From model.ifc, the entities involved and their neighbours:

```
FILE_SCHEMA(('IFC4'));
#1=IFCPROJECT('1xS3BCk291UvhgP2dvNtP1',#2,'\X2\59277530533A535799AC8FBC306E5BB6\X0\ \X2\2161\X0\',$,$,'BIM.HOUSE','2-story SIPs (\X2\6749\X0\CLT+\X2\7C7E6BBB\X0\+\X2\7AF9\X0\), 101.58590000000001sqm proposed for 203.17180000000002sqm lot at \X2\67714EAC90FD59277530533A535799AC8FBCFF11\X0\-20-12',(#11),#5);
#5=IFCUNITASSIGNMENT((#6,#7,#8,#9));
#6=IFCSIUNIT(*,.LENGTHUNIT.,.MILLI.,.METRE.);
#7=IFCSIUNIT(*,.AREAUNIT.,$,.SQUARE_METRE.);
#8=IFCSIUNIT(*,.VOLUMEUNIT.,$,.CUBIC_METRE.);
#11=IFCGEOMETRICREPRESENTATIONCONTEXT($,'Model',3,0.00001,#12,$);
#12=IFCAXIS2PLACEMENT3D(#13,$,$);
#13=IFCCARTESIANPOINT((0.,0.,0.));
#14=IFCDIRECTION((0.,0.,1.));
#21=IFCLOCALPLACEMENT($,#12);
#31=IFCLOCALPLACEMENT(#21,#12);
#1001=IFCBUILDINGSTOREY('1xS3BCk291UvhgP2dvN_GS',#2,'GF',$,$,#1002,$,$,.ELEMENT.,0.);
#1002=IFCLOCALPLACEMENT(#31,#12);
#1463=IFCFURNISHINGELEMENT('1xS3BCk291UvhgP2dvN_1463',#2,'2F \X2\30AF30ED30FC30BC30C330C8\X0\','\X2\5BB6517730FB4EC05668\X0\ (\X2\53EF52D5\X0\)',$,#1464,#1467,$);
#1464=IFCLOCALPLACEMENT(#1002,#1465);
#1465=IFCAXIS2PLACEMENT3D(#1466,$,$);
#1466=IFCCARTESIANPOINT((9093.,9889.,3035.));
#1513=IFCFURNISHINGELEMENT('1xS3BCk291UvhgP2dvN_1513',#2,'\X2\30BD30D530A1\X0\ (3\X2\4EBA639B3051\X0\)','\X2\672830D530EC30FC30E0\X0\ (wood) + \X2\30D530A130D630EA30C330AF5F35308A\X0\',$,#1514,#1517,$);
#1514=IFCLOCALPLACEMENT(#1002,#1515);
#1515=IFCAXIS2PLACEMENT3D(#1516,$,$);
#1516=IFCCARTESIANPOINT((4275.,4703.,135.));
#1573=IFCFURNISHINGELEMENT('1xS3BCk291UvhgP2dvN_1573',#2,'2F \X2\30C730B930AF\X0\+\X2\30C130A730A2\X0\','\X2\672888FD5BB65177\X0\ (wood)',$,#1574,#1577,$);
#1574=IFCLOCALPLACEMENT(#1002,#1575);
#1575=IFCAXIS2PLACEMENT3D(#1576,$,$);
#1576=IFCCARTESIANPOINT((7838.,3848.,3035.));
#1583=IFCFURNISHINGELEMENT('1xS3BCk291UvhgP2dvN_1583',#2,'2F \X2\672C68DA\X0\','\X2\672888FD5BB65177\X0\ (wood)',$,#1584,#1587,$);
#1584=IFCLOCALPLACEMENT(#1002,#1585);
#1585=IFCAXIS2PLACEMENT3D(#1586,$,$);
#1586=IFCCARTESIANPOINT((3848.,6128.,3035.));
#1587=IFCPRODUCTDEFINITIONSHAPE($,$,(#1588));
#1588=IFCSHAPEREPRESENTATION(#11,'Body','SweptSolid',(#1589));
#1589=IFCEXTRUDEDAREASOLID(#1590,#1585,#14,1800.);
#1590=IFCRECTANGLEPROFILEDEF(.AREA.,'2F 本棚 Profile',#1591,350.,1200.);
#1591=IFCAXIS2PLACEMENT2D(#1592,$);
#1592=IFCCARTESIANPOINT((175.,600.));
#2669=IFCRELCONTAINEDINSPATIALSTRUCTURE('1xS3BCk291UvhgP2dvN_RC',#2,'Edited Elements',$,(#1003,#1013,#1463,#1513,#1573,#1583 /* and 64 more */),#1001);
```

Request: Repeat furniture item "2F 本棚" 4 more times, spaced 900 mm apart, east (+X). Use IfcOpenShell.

```python
import numpy as np
import ifcopenshell
import ifcopenshell.api.geometry
import ifcopenshell.api.root
import ifcopenshell.util.element
import ifcopenshell.util.placement

model = ifcopenshell.open("model.ifc")


def reuse_history(source, copy):
    """copy_class also copies each property set's owner history, people and application; keep the originals."""
    for rel in copy.IsDefinedBy:
        if rel.is_a("IfcRelDefinesByProperties") and (history := rel.RelatingPropertyDefinition.OwnerHistory):
            rel.RelatingPropertyDefinition.OwnerHistory = source.OwnerHistory
            ifcopenshell.util.element.remove_deep2(model, history)


source = model.by_guid("1xS3BCk291UvhgP2dvN_1583")
base = ifcopenshell.util.placement.get_local_placement(source.ObjectPlacement)
step = np.array([1.0, 0.0, 0.0]) * 900.0

for i in range(1, 5):
    copy = ifcopenshell.api.root.copy_class(model, product=source)
    copy.Representation = ifcopenshell.util.element.copy_deep(
        model, source.Representation, exclude=["IfcGeometricRepresentationContext", "IfcRepresentationMap"]
    )
    reuse_history(source, copy)
    matrix = base.copy()
    matrix[:3, 3] += i * step
    print("added at", matrix[:3, 3].round(3) + 0.0)
    ifcopenshell.api.geometry.edit_object_placement(model, product=copy, matrix=matrix, is_si=False)

model.write("model_rev.ifc")
```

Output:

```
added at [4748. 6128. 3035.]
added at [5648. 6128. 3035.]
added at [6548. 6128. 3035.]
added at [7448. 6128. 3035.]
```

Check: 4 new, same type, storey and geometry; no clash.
